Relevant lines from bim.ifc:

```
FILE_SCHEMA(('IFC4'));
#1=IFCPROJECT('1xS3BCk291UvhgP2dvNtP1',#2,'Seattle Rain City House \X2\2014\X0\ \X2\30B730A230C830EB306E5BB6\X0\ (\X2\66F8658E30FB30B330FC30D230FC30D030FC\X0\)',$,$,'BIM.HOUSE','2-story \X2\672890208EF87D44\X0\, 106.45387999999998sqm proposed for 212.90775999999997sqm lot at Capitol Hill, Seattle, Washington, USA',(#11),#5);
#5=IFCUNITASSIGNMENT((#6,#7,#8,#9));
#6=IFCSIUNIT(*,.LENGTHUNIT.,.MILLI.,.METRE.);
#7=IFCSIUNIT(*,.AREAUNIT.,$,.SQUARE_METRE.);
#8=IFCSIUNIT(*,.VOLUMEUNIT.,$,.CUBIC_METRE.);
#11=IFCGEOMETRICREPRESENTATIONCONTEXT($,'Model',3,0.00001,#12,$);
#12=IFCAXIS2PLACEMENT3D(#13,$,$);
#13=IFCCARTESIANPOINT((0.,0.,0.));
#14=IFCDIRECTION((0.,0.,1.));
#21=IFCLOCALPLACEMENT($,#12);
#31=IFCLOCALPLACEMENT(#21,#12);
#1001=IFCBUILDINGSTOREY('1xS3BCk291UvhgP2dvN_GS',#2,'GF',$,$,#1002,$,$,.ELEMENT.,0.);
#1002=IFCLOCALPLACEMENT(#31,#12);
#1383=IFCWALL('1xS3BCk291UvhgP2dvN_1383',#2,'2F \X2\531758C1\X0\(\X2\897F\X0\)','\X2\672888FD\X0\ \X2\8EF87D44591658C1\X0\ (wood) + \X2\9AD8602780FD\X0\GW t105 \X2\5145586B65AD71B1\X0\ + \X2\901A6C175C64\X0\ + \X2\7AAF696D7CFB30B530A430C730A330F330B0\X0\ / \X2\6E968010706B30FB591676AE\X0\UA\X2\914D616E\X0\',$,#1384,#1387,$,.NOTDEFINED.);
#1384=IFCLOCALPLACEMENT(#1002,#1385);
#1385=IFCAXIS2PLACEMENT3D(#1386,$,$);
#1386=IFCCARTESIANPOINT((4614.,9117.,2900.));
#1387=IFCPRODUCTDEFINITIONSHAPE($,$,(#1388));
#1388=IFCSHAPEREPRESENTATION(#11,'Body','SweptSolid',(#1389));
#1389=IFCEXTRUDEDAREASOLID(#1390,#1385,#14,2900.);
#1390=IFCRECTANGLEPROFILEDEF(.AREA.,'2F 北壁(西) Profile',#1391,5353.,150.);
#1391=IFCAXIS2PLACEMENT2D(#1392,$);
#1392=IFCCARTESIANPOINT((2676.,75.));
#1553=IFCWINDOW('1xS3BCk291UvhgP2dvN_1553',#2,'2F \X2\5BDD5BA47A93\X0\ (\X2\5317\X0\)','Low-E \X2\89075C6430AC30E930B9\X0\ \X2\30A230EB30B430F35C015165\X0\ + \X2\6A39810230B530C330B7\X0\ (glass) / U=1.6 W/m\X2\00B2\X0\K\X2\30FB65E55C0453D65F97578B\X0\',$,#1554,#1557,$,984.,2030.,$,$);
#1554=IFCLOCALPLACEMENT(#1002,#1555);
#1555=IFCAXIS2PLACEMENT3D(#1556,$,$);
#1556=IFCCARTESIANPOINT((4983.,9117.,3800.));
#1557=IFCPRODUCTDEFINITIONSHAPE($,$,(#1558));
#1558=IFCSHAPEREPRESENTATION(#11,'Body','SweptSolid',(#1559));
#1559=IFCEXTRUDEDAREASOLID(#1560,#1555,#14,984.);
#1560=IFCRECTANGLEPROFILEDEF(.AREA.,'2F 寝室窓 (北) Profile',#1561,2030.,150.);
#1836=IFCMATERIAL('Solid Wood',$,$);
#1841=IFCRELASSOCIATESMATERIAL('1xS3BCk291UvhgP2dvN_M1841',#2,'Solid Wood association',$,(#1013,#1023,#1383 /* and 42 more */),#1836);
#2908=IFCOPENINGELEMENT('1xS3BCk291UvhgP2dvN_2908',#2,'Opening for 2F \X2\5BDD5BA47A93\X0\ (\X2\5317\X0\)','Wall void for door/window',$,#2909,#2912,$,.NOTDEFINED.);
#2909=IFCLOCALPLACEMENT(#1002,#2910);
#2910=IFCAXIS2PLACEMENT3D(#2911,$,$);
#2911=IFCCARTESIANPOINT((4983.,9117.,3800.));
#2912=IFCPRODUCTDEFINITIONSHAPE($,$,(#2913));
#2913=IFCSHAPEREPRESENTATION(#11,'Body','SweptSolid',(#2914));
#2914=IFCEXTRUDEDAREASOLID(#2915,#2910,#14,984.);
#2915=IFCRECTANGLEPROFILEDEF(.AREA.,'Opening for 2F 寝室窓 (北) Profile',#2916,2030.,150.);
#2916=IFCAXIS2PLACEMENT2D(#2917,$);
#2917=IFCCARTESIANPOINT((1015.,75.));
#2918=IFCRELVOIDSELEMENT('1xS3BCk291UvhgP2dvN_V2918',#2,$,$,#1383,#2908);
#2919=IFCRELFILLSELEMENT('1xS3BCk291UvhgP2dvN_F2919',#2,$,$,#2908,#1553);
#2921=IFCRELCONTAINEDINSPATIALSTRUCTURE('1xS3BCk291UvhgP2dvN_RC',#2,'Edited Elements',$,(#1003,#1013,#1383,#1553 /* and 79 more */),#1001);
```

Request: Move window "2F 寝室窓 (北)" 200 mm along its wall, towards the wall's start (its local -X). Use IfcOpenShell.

```python
import ifcopenshell
import ifcopenshell.api.geometry
import ifcopenshell.util.placement
import ifcopenshell.util.unit

model = ifcopenshell.open("bim.ifc")
unit_scale = ifcopenshell.util.unit.calculate_unit_scale(model)

window = model.by_guid("1xS3BCk291UvhgP2dvN_1553")
opening = window.FillsVoids[0].RelatingOpeningElement
wall = opening.VoidsElements[0].RelatingBuildingElement

wall_matrix = ifcopenshell.util.placement.get_local_placement(wall.ObjectPlacement)
shift = wall_matrix[:3, 0] * -0.2 / unit_scale
before = ifcopenshell.util.placement.get_local_placement(window.ObjectPlacement)[:3, 3].copy()

# The window is not placed relative to its opening, so move both.
for product in (opening, window):
    matrix = ifcopenshell.util.placement.get_local_placement(product.ObjectPlacement)
    matrix[:3, 3] += shift
    ifcopenshell.api.geometry.edit_object_placement(model, product=product, matrix=matrix, is_si=False)

after = ifcopenshell.util.placement.get_local_placement(window.ObjectPlacement)[:3, 3]
print("window moved by", (after - before).round(3) + 0.0)

model.write("bim_v2.ifc")
```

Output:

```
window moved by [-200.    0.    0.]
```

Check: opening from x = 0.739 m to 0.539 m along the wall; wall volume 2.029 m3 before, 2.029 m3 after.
